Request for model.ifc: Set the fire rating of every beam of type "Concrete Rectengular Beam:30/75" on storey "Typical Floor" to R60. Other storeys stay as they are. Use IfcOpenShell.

First a look at what the model holds.

```python
import ifcopenshell
import ifcopenshell.util.element

model = ifcopenshell.open("model.ifc")
print(model.schema)
storey = next(s for s in model.by_type("IfcBuildingStorey") if s.Name == "Typical Floor")
beams = [e for e in ifcopenshell.util.element.get_decomposition(storey) if e.is_a("IfcBeam")]
seen = {}
for e in beams:
    element_type = ifcopenshell.util.element.get_type(e)
    key = (element_type.Name if element_type != e and element_type else None, ifcopenshell.util.element.get_pset(e, "Pset_BeamCommon", "FireRating"))
    seen[key] = seen.get(key, 0) + 1
for (name, value), count in sorted(seen.items(), key=str):
    print(count, "x", name, "|", value)
```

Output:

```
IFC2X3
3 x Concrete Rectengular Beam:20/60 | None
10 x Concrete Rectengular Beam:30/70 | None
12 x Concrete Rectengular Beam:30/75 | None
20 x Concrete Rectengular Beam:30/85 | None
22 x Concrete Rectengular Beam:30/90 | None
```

```python
import ifcopenshell
import ifcopenshell.api.pset
import ifcopenshell.util.element

model = ifcopenshell.open("model.ifc")

storey = next(s for s in model.by_type("IfcBuildingStorey") if s.Name == "Typical Floor")
beams = [e for e in ifcopenshell.util.element.get_decomposition(storey) if e.is_a("IfcBeam")]

count = 0
for e in beams:
    element_type = ifcopenshell.util.element.get_type(e)
    if element_type in (None, e) or element_type.Name != "Concrete Rectengular Beam:30/75":
        continue
    # add_pset returns the element's existing set when there is one.
    pset = ifcopenshell.api.pset.add_pset(model, product=e, name="Pset_BeamCommon")
    ifcopenshell.api.pset.edit_pset(model, pset=pset, properties={"FireRating": "R60"})
    count += 1

print(count, "beams updated")

model.write("model_v2.ifc")
```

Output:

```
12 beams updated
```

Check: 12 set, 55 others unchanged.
